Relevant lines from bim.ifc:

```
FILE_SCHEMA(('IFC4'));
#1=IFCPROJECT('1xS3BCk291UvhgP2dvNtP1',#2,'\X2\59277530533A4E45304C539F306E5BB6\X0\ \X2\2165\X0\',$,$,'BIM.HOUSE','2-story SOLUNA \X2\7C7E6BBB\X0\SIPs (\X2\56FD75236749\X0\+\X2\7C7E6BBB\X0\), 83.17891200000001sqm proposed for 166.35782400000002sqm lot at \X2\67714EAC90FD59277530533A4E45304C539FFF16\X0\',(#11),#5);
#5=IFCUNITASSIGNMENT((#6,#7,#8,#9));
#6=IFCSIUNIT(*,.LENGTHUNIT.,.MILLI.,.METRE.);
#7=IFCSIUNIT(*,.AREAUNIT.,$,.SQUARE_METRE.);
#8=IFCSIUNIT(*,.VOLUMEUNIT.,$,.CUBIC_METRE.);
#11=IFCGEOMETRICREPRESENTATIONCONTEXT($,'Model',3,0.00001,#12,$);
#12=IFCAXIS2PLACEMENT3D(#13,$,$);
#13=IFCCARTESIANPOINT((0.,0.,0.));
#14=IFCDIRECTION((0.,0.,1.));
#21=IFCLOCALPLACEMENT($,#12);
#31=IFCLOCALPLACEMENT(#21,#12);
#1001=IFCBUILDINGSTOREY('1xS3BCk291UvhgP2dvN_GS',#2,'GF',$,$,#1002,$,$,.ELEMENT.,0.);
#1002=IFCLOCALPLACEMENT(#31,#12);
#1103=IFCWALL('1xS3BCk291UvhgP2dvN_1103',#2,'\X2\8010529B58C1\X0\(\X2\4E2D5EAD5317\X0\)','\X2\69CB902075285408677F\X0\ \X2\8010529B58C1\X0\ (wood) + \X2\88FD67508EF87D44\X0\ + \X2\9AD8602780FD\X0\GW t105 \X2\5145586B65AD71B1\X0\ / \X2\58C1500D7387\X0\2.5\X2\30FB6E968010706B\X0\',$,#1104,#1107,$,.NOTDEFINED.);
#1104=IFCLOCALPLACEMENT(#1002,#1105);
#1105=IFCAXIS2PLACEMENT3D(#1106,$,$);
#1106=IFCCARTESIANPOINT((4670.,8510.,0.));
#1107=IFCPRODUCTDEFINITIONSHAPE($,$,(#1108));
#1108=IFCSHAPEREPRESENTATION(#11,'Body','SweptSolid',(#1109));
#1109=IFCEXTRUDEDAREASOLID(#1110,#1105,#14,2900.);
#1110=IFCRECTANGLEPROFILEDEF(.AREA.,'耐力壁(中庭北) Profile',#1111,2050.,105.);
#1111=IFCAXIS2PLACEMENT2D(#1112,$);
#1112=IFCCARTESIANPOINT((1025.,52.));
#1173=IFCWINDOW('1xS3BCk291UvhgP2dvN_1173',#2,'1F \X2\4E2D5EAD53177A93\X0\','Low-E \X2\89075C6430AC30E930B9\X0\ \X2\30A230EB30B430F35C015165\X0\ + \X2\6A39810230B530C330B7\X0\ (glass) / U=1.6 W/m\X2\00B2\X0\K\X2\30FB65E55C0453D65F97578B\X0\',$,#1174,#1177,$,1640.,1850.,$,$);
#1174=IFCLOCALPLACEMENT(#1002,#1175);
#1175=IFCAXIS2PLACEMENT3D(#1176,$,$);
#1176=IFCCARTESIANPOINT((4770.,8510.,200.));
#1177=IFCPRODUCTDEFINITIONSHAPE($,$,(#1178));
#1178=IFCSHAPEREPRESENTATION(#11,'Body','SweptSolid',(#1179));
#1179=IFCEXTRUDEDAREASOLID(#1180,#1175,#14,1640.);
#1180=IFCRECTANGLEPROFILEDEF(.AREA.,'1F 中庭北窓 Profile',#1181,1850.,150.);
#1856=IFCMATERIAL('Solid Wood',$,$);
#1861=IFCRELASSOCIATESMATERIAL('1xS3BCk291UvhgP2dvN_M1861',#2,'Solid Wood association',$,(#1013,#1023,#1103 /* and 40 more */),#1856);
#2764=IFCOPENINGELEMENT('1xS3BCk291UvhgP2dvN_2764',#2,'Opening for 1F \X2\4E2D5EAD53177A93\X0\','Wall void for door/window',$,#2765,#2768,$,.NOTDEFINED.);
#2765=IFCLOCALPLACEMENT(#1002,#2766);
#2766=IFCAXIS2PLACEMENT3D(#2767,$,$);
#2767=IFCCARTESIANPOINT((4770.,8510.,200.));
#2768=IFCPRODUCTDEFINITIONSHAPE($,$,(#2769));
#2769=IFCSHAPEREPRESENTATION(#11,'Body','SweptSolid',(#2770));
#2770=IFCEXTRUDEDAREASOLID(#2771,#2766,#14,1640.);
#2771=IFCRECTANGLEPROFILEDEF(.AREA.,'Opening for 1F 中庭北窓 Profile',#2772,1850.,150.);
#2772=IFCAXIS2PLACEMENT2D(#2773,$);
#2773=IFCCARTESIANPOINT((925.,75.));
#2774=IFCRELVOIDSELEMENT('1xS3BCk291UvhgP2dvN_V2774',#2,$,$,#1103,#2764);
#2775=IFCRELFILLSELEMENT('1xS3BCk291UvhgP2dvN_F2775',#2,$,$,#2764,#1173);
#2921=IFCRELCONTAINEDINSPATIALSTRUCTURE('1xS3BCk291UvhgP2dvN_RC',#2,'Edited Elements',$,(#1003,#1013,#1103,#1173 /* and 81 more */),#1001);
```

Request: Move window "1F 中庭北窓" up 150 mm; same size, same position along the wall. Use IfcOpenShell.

```python
import numpy as np
import ifcopenshell
import ifcopenshell.api.geometry
import ifcopenshell.util.placement
import ifcopenshell.util.unit

model = ifcopenshell.open("bim.ifc")
unit_scale = ifcopenshell.util.unit.calculate_unit_scale(model)

window = model.by_guid("1xS3BCk291UvhgP2dvN_1173")
opening = window.FillsVoids[0].RelatingOpeningElement
dz = 0.15 / unit_scale

shift = np.array([0.0, 0.0, dz])
# The window is not placed relative to its opening, so move both.
for product in (opening, window):
    matrix = ifcopenshell.util.placement.get_local_placement(product.ObjectPlacement)
    matrix[:3, 3] += shift
    ifcopenshell.api.geometry.edit_object_placement(model, product=product, matrix=matrix, is_si=False)

print(f"moved by {dz * unit_scale:+.3f} m")

model.write("bim_v2.ifc")
```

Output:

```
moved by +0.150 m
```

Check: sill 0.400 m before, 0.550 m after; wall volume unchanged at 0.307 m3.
